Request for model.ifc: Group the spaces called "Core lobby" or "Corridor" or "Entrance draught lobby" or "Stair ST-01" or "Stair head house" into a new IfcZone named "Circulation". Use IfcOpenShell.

First a look at what the model holds.

```python
import ifcopenshell

model = ifcopenshell.open("model.ifc")
print(model.schema)
seen = {}
for space in model.by_type("IfcSpace"):
    seen[space.LongName] = seen.get(space.LongName, 0) + 1
for name, count in sorted(seen.items(), key=str):
    print(count, "x", name)
print("zones:", [z.Name for z in model.by_type("IfcZone")][:20])
```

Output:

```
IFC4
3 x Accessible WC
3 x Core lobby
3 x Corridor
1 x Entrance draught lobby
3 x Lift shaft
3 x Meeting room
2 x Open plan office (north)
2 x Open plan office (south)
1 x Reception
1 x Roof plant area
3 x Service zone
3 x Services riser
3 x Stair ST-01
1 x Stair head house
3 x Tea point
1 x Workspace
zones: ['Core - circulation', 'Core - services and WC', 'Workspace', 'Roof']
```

```python
import ifcopenshell
import ifcopenshell.api.group
import ifcopenshell.api.root

model = ifcopenshell.open("model.ifc")

names = {"Core lobby", "Corridor", "Entrance draught lobby", "Stair ST-01", "Stair head house"}
spaces = [s for s in model.by_type("IfcSpace") if s.LongName in names]

zone = ifcopenshell.api.root.create_entity(model, ifc_class="IfcZone", name="Circulation")
ifcopenshell.api.group.assign_group(model, products=spaces, group=zone)
print(len(spaces), "spaces in", zone.Name)

model.write("model_v2.ifc")
```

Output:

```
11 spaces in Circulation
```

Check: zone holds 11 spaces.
